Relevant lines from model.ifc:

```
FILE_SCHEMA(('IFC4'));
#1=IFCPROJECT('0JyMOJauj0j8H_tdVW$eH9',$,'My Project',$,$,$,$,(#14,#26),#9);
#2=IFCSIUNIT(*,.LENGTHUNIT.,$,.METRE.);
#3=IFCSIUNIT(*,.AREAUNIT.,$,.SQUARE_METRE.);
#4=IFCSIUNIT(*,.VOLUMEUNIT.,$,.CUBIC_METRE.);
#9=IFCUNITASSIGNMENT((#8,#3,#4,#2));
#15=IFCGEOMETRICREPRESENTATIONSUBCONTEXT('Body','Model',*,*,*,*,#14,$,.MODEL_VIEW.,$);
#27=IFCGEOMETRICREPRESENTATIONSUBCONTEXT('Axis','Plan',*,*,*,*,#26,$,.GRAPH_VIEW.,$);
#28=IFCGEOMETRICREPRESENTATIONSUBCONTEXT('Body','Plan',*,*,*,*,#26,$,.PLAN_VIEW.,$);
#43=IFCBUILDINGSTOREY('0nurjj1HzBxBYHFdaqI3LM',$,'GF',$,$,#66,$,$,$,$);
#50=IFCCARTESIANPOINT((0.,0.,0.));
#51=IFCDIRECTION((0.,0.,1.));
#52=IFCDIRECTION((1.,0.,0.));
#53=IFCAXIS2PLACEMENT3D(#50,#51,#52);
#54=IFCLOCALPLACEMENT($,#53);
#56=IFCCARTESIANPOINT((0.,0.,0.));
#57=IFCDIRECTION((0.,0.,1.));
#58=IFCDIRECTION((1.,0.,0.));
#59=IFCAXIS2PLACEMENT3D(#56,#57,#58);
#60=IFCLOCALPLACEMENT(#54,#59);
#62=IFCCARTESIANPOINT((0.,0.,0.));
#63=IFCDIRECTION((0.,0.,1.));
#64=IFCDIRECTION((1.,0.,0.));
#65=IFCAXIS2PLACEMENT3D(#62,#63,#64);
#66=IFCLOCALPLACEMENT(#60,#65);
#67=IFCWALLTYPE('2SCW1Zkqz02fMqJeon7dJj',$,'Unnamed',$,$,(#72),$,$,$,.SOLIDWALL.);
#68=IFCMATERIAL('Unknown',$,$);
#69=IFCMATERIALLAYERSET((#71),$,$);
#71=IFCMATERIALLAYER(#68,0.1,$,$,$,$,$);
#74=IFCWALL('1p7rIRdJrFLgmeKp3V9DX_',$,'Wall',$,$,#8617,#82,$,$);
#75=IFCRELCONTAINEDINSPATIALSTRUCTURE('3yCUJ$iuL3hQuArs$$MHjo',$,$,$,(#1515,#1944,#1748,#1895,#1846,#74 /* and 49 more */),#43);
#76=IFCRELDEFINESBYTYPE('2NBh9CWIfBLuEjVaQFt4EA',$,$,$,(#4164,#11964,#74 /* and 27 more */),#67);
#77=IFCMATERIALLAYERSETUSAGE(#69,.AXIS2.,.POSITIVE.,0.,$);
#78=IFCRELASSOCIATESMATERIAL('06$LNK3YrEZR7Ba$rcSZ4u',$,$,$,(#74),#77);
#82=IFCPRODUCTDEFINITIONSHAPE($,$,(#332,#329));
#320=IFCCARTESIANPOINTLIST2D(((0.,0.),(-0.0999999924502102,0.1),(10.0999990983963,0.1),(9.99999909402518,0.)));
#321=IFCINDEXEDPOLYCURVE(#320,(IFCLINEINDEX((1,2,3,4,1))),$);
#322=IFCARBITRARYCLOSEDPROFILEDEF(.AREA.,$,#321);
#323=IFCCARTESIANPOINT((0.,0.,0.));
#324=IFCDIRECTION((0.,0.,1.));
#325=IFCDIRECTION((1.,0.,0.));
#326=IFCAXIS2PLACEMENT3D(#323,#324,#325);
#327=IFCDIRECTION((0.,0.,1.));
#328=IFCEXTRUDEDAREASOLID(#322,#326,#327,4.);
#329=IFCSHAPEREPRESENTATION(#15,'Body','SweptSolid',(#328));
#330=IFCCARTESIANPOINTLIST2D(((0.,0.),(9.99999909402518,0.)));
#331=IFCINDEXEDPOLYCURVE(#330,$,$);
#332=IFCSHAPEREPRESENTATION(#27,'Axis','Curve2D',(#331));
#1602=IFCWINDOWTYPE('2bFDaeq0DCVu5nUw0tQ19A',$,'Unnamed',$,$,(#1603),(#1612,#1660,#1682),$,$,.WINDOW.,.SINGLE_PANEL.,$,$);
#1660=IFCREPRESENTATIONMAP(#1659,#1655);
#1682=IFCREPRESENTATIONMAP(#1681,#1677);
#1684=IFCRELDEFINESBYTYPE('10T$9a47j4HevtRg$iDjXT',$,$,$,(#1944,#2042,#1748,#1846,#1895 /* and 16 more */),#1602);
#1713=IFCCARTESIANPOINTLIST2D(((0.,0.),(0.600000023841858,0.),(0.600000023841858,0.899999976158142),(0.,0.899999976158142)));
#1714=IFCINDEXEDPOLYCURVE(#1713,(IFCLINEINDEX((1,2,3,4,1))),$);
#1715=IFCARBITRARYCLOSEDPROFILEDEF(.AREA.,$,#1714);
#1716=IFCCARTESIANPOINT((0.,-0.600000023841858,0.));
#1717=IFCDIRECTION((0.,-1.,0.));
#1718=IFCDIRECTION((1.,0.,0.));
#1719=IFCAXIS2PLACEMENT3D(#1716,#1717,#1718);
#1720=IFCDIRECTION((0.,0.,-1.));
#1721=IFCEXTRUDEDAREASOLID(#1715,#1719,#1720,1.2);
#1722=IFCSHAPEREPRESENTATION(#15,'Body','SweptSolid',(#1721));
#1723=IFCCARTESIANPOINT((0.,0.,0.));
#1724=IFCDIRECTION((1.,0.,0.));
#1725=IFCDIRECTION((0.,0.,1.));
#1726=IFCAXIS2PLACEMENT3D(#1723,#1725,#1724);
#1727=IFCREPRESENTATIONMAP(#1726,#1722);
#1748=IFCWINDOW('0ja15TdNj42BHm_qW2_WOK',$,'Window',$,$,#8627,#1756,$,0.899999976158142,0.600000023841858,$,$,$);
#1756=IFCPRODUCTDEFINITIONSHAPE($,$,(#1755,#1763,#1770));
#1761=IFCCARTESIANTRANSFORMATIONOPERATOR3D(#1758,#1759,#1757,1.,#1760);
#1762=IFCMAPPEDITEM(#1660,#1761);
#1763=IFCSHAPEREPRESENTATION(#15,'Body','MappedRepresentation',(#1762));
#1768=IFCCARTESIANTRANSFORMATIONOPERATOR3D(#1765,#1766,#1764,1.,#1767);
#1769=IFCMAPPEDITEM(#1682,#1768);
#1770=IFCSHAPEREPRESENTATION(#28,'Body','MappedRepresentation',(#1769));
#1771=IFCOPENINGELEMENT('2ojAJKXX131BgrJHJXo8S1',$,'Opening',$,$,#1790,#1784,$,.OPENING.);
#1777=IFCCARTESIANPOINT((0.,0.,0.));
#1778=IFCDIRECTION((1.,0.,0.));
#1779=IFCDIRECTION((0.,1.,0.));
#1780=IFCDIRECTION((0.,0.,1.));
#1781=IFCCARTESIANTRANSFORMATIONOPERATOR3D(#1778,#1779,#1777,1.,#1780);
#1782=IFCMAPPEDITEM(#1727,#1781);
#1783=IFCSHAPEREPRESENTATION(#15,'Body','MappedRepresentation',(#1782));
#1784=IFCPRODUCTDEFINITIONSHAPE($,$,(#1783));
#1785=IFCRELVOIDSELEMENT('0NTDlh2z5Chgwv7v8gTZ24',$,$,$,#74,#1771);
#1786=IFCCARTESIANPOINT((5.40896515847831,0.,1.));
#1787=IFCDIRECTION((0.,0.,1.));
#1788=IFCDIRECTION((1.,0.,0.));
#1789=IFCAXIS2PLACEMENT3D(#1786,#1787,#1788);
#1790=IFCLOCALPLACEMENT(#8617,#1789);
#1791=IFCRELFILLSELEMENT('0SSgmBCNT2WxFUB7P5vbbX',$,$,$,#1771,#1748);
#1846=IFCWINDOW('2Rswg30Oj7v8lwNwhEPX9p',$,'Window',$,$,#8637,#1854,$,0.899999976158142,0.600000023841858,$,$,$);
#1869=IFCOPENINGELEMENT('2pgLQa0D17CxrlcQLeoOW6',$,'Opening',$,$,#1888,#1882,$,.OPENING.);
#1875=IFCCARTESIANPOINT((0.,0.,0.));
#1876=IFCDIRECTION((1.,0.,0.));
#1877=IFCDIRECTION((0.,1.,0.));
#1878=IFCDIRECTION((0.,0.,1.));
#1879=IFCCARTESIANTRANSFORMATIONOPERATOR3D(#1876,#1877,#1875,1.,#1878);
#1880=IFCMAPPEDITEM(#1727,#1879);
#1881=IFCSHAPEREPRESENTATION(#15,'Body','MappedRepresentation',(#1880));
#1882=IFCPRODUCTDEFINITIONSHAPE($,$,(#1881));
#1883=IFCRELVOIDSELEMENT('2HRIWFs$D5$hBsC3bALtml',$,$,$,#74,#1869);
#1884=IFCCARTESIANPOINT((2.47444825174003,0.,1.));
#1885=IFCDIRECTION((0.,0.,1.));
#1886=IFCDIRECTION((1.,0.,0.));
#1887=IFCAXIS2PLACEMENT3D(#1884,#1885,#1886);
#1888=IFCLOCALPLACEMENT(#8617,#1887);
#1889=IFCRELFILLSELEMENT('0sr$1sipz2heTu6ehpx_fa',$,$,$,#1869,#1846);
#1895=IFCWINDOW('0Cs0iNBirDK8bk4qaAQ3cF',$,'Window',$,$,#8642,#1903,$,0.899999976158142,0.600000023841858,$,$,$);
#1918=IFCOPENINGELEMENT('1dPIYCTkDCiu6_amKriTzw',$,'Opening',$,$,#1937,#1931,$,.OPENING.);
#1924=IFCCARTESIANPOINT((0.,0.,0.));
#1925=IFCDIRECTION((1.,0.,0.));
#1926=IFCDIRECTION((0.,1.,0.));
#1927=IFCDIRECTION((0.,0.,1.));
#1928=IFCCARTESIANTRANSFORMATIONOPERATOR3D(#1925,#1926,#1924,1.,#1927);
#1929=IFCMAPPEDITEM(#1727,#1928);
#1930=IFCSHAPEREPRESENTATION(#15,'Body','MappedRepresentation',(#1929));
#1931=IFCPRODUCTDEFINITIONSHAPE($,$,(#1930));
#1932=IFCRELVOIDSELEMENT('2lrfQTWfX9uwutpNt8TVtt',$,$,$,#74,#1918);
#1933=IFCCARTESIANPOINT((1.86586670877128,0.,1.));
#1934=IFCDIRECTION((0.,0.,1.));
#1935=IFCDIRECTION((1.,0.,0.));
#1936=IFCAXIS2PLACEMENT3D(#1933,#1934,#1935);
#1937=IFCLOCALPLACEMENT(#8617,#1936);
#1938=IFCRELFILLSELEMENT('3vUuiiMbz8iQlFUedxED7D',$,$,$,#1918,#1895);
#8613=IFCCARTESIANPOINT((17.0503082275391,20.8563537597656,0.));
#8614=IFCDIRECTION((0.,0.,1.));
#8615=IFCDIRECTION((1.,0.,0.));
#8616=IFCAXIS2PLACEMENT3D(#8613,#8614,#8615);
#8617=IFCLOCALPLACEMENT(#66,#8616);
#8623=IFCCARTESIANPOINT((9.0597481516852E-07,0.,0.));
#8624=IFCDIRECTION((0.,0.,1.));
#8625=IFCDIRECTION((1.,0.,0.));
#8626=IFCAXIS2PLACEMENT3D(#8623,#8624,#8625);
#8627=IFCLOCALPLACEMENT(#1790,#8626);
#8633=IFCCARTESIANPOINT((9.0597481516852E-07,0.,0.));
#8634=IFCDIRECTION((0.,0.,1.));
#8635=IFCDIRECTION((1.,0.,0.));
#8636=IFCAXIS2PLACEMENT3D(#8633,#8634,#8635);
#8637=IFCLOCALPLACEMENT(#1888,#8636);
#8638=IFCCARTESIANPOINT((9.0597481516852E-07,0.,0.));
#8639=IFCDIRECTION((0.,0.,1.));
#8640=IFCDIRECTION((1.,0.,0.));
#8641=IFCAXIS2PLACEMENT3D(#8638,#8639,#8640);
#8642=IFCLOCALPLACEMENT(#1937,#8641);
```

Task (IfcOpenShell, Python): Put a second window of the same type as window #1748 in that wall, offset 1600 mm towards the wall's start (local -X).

```python
import ifcopenshell
import ifcopenshell.api.feature
import ifcopenshell.api.geometry
import ifcopenshell.api.root
import ifcopenshell.geom
import ifcopenshell.util.element
import ifcopenshell.util.placement
import ifcopenshell.util.shape
import ifcopenshell.util.unit

model = ifcopenshell.open("model.ifc")
unit_scale = ifcopenshell.util.unit.calculate_unit_scale(model)
settings = ifcopenshell.geom.settings()


def volume(element):
    """Net volume in cubic metres, openings subtracted."""
    shape = ifcopenshell.geom.create_shape(settings, element)
    return ifcopenshell.util.shape.get_volume(shape.geometry)


window = model.by_guid("0ja15TdNj42BHm_qW2_WOK")
opening = window.FillsVoids[0].RelatingOpeningElement
wall = opening.VoidsElements[0].RelatingBuildingElement
before = volume(wall)
shift = ifcopenshell.util.placement.get_local_placement(wall.ObjectPlacement)[:3, 0] * -1.6 / unit_scale

# copy_class copies the void relationship, type, container and properties, but no geometry.
new_opening = ifcopenshell.api.root.copy_class(model, product=opening)
new_opening.Representation = ifcopenshell.util.element.copy_deep(
    model, opening.Representation, exclude=["IfcGeometricRepresentationContext", "IfcRepresentationMap"]
)
new_window = ifcopenshell.api.root.copy_class(model, product=window)
new_window.Representation = ifcopenshell.util.element.copy_deep(
    model, window.Representation, exclude=["IfcGeometricRepresentationContext", "IfcRepresentationMap"]
)
ifcopenshell.api.feature.add_filling(model, opening=new_opening, element=new_window)

for old, new in ((opening, new_opening), (window, new_window)):
    matrix = ifcopenshell.util.placement.get_local_placement(old.ObjectPlacement)
    matrix[:3, 3] += shift
    ifcopenshell.api.geometry.edit_object_placement(model, product=new, matrix=matrix, is_si=False)

after = volume(wall)

print(f"wall volume {before:.3f} -> {after:.3f} m3")

model.write("model_rev.ifc")
```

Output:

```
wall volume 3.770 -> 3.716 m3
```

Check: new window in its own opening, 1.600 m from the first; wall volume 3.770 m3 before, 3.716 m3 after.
